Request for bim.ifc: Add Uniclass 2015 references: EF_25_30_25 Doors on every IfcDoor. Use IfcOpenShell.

First a look at what the model holds.

```python
import ifcopenshell

model = ifcopenshell.open("bim.ifc")
print(model.schema)
print("classifications:", [c.Name for c in model.by_type("IfcClassification")])
for ifc_class in ("IfcDoor", "IfcRoof", "IfcStair", "IfcWall", "IfcWindow"):
    print(ifc_class, len(model.by_type(ifc_class)))
```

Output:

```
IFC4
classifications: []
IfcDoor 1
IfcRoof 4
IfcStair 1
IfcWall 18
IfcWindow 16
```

```python
import ifcopenshell
import ifcopenshell.api.classification

model = ifcopenshell.open("bim.ifc")

system = ifcopenshell.api.classification.add_classification(model, classification="Uniclass 2015")

codes = {
    "IfcDoor": ("EF_25_30_25", "Doors"),
}
for ifc_class, (code, name) in codes.items():
    products = model.by_type(ifc_class)
    ifcopenshell.api.classification.add_reference(
        model, products=products, classification=system, identification=code, name=name
    )
    print(code, len(products))

model.write("bim_edited.ifc")
```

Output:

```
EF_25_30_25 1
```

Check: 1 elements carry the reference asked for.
